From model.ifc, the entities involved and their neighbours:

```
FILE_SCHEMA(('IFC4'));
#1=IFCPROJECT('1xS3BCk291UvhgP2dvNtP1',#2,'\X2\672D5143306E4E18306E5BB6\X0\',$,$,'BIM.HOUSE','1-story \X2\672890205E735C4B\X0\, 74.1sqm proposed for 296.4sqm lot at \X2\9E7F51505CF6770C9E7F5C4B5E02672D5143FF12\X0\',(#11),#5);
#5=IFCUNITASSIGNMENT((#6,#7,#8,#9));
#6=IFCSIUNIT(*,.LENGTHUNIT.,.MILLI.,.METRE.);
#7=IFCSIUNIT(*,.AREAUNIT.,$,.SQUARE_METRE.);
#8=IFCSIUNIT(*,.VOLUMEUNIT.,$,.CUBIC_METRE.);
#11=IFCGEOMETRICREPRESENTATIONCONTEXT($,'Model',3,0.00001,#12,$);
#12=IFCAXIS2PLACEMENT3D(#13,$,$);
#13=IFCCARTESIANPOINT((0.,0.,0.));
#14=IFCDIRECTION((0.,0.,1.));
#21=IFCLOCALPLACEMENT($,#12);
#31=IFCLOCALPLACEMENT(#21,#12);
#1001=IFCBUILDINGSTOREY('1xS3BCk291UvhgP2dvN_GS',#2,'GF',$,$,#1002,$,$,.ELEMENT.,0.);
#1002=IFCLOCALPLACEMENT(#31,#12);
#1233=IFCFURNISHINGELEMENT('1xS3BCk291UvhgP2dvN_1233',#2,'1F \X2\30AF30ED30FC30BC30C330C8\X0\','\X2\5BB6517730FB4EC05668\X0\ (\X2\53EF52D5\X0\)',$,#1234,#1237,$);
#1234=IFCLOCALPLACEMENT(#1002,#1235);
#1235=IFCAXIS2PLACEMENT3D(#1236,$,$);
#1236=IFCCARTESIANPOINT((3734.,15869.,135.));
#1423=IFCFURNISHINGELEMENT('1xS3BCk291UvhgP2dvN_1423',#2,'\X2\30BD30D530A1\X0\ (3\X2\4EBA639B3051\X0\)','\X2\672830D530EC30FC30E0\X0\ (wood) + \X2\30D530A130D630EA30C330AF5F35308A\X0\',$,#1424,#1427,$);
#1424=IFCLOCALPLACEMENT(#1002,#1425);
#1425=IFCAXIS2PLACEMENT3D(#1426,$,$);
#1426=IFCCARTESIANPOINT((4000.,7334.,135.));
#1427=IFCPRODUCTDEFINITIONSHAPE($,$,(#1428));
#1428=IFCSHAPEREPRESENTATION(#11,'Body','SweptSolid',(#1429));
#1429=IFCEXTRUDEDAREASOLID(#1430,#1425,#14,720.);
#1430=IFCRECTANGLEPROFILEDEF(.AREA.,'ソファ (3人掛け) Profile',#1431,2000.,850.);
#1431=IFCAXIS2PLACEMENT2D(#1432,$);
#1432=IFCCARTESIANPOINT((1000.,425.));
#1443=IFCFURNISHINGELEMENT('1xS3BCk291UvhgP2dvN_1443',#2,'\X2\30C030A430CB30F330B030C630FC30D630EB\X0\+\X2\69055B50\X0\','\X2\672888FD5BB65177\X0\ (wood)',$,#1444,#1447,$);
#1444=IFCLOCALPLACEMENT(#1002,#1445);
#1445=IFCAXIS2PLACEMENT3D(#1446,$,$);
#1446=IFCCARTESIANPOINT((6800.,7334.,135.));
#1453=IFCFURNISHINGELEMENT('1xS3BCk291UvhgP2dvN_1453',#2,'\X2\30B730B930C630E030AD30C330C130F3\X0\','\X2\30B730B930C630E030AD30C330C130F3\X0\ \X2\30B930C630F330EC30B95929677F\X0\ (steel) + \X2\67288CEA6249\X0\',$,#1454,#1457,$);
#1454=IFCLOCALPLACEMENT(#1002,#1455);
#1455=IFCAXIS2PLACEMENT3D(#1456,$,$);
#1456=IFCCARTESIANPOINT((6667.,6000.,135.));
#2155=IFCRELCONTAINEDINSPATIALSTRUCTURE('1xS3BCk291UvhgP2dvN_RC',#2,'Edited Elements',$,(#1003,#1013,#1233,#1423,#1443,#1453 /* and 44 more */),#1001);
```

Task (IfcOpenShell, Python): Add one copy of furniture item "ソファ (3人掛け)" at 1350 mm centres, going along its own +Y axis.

```python
import ifcopenshell
import ifcopenshell.api.geometry
import ifcopenshell.api.root
import ifcopenshell.util.element
import ifcopenshell.util.placement
import ifcopenshell.util.unit

model = ifcopenshell.open("model.ifc")
unit_scale = ifcopenshell.util.unit.calculate_unit_scale(model)


def reuse_history(source, copy):
    """copy_class also copies each property set's owner history, people and application; keep the originals."""
    for rel in copy.IsDefinedBy:
        if rel.is_a("IfcRelDefinesByProperties") and (history := rel.RelatingPropertyDefinition.OwnerHistory):
            rel.RelatingPropertyDefinition.OwnerHistory = source.OwnerHistory
            ifcopenshell.util.element.remove_deep2(model, history)


source = model.by_guid("1xS3BCk291UvhgP2dvN_1423")
base = ifcopenshell.util.placement.get_local_placement(source.ObjectPlacement)
step = base[:3, 1] * 1.35 / unit_scale

for i in range(1, 2):
    copy = ifcopenshell.api.root.copy_class(model, product=source)
    copy.Representation = ifcopenshell.util.element.copy_deep(
        model, source.Representation, exclude=["IfcGeometricRepresentationContext", "IfcRepresentationMap"]
    )
    reuse_history(source, copy)
    matrix = base.copy()
    matrix[:3, 3] += i * step
    print("added at", matrix[:3, 3].round(3) + 0.0)
    ifcopenshell.api.geometry.edit_object_placement(model, product=copy, matrix=matrix, is_si=False)

model.write("model_rev.ifc")
```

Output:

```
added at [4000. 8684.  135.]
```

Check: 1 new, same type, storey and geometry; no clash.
